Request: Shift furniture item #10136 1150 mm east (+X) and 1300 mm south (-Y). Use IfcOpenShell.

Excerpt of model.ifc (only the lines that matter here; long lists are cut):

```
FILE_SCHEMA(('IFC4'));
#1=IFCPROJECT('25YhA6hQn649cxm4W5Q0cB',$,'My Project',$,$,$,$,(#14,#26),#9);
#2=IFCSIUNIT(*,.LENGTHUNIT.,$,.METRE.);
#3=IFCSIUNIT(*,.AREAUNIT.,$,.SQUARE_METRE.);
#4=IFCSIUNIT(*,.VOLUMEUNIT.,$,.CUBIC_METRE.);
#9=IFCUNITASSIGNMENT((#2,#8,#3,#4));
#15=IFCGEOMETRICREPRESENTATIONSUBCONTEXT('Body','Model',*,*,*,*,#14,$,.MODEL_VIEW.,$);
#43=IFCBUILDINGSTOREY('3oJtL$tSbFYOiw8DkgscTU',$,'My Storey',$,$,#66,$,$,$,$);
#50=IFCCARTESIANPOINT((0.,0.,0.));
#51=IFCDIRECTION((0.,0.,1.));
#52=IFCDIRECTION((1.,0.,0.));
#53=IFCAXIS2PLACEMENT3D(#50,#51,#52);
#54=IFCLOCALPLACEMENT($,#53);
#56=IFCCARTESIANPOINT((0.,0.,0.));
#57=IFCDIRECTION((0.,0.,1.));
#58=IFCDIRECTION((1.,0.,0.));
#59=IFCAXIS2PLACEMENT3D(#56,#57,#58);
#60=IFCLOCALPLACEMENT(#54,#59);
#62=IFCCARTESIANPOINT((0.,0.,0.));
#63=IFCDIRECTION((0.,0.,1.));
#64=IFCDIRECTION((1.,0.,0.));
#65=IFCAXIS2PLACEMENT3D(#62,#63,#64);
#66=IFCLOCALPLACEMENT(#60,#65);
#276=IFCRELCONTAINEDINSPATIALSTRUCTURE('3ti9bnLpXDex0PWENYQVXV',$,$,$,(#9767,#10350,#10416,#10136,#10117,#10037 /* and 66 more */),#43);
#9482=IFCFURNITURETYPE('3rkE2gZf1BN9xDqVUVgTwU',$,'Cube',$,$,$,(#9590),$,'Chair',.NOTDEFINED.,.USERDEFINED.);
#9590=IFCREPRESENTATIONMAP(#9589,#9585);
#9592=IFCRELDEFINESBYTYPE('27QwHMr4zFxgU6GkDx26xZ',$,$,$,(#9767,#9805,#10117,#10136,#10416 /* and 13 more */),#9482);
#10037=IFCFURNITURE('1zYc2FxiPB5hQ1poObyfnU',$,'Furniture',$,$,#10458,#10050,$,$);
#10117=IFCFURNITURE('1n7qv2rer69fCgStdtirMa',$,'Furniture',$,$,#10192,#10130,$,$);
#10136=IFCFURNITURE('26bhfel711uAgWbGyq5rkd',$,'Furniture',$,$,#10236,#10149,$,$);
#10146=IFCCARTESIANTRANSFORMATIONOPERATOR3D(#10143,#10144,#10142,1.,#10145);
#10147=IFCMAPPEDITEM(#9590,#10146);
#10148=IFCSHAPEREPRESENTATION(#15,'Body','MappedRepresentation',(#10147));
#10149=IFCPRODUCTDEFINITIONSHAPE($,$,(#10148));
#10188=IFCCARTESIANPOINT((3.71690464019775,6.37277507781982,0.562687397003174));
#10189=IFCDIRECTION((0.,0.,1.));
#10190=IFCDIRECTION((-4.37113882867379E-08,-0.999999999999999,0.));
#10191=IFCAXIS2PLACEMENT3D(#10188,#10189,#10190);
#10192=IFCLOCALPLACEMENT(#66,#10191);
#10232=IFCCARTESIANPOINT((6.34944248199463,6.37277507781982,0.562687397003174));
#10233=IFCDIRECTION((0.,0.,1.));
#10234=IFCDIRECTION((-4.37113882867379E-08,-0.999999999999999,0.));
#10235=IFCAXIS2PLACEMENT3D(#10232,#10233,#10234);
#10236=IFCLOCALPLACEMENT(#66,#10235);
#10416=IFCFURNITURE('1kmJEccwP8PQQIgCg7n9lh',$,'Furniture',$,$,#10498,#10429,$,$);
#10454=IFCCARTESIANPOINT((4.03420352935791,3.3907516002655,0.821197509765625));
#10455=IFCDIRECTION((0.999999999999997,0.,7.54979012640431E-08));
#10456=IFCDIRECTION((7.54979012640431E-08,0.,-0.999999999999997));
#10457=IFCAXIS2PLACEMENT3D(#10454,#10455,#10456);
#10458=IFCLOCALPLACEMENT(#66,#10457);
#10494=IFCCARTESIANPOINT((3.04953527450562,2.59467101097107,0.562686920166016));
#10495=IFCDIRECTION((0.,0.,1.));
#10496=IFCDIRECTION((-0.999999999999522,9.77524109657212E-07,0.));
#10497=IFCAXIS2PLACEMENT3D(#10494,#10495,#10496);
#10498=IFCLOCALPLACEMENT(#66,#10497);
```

```python
import ifcopenshell
import ifcopenshell.api.geometry
import ifcopenshell.util.placement

model = ifcopenshell.open("model.ifc")

item = model.by_guid("26bhfel711uAgWbGyq5rkd")
matrix = ifcopenshell.util.placement.get_local_placement(item.ObjectPlacement)
matrix[0, 3] += 1.15
matrix[1, 3] -= 1.3
ifcopenshell.api.geometry.edit_object_placement(model, product=item, matrix=matrix, is_si=False)

print(ifcopenshell.util.placement.get_local_placement(item.ObjectPlacement).round(3) + 0.0)

model.write("model_v2.ifc")
```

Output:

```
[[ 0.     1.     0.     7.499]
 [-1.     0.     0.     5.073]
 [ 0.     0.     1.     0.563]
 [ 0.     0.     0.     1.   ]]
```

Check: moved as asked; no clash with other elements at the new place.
